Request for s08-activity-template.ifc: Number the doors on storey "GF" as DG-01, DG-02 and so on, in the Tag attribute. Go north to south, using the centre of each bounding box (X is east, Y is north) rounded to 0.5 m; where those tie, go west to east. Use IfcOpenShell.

First a look at what the model holds.

```python
import ifcopenshell
import ifcopenshell.util.element
import ifcopenshell.util.placement

model = ifcopenshell.open("s08-activity-template.ifc")
print(model.schema)
storey = next(s for s in model.by_type("IfcBuildingStorey") if s.Name == "GF")
doors = [e for e in ifcopenshell.util.element.get_decomposition(storey) if e.is_a("IfcDoor")]
for e in sorted(doors, key=lambda e: e.id()):
    origin = ifcopenshell.util.placement.get_local_placement(e.ObjectPlacement)[:3, 3]
    print(e.id(), e.Tag, e.Name, origin.round(2) + 0.0, sep=" | ")
```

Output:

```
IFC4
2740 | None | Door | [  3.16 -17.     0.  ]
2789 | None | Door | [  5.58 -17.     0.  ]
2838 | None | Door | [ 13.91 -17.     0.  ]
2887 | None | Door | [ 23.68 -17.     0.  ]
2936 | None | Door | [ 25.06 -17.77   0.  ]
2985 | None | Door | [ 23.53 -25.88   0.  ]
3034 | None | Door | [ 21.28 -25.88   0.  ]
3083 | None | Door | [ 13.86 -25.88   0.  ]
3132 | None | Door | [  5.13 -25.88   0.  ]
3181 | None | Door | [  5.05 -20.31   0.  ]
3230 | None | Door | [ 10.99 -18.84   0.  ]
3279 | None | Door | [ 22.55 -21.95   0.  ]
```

```python
import ifcopenshell
import ifcopenshell.geom
import ifcopenshell.util.element
import ifcopenshell.util.shape

model = ifcopenshell.open("s08-activity-template.ifc")
settings = ifcopenshell.geom.settings()
settings.set("use-world-coords", True)


def centre(element):
    shape = ifcopenshell.geom.create_shape(settings, element)
    return ifcopenshell.util.shape.get_bbox_centroid(shape.geometry)


storey = next(s for s in model.by_type("IfcBuildingStorey") if s.Name == "GF")
doors = [e for e in ifcopenshell.util.element.get_decomposition(storey) if e.is_a("IfcDoor")]

# Insertion points can sit at a corner or the storey origin, so sort by the geometry (in metres).
centres = {e: centre(e) for e in doors}
doors.sort(key=lambda e: (-round(centres[e][1] / 0.5), centres[e][0]))

for i, e in enumerate(doors, start=1):
    number = f"DG-{i:02d}"
    e.Tag = number
    print(e.id(), number)

model.write("s08-activity-template_updated.ifc")
```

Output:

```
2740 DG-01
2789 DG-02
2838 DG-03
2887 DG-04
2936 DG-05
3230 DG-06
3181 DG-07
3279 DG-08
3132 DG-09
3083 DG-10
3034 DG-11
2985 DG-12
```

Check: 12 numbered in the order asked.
